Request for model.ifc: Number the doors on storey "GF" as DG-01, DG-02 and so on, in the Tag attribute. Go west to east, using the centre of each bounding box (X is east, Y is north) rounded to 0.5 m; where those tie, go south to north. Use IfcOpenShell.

First a look at what the model holds.

```python
import ifcopenshell
import ifcopenshell.util.element
import ifcopenshell.util.placement

model = ifcopenshell.open("model.ifc")
print(model.schema)
storey = next(s for s in model.by_type("IfcBuildingStorey") if s.Name == "GF")
doors = [e for e in ifcopenshell.util.element.get_decomposition(storey) if e.is_a("IfcDoor")]
for e in sorted(doors, key=lambda e: e.id()):
    origin = ifcopenshell.util.placement.get_local_placement(e.ObjectPlacement)[:3, 3]
    print(e.id(), e.Tag, e.Name, origin.round(2) + 0.0, sep=" | ")
```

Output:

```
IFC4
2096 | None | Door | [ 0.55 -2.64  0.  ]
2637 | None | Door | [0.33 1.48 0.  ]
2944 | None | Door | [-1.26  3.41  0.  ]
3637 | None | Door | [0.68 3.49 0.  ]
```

```python
import ifcopenshell
import ifcopenshell.geom
import ifcopenshell.util.element
import ifcopenshell.util.shape

model = ifcopenshell.open("model.ifc")
settings = ifcopenshell.geom.settings()
settings.set("use-world-coords", True)


def centre(element):
    shape = ifcopenshell.geom.create_shape(settings, element)
    return ifcopenshell.util.shape.get_bbox_centroid(shape.geometry)


storey = next(s for s in model.by_type("IfcBuildingStorey") if s.Name == "GF")
doors = [e for e in ifcopenshell.util.element.get_decomposition(storey) if e.is_a("IfcDoor")]

# Insertion points can sit at a corner or the storey origin, so sort by the geometry (in metres).
centres = {e: centre(e) for e in doors}
doors.sort(key=lambda e: (round(centres[e][0] / 0.5), centres[e][1]))

for i, e in enumerate(doors, start=1):
    number = f"DG-{i:02d}"
    e.Tag = number
    print(e.id(), number)

model.write("model_rev.ifc")
```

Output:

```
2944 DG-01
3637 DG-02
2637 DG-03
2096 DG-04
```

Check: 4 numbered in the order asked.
